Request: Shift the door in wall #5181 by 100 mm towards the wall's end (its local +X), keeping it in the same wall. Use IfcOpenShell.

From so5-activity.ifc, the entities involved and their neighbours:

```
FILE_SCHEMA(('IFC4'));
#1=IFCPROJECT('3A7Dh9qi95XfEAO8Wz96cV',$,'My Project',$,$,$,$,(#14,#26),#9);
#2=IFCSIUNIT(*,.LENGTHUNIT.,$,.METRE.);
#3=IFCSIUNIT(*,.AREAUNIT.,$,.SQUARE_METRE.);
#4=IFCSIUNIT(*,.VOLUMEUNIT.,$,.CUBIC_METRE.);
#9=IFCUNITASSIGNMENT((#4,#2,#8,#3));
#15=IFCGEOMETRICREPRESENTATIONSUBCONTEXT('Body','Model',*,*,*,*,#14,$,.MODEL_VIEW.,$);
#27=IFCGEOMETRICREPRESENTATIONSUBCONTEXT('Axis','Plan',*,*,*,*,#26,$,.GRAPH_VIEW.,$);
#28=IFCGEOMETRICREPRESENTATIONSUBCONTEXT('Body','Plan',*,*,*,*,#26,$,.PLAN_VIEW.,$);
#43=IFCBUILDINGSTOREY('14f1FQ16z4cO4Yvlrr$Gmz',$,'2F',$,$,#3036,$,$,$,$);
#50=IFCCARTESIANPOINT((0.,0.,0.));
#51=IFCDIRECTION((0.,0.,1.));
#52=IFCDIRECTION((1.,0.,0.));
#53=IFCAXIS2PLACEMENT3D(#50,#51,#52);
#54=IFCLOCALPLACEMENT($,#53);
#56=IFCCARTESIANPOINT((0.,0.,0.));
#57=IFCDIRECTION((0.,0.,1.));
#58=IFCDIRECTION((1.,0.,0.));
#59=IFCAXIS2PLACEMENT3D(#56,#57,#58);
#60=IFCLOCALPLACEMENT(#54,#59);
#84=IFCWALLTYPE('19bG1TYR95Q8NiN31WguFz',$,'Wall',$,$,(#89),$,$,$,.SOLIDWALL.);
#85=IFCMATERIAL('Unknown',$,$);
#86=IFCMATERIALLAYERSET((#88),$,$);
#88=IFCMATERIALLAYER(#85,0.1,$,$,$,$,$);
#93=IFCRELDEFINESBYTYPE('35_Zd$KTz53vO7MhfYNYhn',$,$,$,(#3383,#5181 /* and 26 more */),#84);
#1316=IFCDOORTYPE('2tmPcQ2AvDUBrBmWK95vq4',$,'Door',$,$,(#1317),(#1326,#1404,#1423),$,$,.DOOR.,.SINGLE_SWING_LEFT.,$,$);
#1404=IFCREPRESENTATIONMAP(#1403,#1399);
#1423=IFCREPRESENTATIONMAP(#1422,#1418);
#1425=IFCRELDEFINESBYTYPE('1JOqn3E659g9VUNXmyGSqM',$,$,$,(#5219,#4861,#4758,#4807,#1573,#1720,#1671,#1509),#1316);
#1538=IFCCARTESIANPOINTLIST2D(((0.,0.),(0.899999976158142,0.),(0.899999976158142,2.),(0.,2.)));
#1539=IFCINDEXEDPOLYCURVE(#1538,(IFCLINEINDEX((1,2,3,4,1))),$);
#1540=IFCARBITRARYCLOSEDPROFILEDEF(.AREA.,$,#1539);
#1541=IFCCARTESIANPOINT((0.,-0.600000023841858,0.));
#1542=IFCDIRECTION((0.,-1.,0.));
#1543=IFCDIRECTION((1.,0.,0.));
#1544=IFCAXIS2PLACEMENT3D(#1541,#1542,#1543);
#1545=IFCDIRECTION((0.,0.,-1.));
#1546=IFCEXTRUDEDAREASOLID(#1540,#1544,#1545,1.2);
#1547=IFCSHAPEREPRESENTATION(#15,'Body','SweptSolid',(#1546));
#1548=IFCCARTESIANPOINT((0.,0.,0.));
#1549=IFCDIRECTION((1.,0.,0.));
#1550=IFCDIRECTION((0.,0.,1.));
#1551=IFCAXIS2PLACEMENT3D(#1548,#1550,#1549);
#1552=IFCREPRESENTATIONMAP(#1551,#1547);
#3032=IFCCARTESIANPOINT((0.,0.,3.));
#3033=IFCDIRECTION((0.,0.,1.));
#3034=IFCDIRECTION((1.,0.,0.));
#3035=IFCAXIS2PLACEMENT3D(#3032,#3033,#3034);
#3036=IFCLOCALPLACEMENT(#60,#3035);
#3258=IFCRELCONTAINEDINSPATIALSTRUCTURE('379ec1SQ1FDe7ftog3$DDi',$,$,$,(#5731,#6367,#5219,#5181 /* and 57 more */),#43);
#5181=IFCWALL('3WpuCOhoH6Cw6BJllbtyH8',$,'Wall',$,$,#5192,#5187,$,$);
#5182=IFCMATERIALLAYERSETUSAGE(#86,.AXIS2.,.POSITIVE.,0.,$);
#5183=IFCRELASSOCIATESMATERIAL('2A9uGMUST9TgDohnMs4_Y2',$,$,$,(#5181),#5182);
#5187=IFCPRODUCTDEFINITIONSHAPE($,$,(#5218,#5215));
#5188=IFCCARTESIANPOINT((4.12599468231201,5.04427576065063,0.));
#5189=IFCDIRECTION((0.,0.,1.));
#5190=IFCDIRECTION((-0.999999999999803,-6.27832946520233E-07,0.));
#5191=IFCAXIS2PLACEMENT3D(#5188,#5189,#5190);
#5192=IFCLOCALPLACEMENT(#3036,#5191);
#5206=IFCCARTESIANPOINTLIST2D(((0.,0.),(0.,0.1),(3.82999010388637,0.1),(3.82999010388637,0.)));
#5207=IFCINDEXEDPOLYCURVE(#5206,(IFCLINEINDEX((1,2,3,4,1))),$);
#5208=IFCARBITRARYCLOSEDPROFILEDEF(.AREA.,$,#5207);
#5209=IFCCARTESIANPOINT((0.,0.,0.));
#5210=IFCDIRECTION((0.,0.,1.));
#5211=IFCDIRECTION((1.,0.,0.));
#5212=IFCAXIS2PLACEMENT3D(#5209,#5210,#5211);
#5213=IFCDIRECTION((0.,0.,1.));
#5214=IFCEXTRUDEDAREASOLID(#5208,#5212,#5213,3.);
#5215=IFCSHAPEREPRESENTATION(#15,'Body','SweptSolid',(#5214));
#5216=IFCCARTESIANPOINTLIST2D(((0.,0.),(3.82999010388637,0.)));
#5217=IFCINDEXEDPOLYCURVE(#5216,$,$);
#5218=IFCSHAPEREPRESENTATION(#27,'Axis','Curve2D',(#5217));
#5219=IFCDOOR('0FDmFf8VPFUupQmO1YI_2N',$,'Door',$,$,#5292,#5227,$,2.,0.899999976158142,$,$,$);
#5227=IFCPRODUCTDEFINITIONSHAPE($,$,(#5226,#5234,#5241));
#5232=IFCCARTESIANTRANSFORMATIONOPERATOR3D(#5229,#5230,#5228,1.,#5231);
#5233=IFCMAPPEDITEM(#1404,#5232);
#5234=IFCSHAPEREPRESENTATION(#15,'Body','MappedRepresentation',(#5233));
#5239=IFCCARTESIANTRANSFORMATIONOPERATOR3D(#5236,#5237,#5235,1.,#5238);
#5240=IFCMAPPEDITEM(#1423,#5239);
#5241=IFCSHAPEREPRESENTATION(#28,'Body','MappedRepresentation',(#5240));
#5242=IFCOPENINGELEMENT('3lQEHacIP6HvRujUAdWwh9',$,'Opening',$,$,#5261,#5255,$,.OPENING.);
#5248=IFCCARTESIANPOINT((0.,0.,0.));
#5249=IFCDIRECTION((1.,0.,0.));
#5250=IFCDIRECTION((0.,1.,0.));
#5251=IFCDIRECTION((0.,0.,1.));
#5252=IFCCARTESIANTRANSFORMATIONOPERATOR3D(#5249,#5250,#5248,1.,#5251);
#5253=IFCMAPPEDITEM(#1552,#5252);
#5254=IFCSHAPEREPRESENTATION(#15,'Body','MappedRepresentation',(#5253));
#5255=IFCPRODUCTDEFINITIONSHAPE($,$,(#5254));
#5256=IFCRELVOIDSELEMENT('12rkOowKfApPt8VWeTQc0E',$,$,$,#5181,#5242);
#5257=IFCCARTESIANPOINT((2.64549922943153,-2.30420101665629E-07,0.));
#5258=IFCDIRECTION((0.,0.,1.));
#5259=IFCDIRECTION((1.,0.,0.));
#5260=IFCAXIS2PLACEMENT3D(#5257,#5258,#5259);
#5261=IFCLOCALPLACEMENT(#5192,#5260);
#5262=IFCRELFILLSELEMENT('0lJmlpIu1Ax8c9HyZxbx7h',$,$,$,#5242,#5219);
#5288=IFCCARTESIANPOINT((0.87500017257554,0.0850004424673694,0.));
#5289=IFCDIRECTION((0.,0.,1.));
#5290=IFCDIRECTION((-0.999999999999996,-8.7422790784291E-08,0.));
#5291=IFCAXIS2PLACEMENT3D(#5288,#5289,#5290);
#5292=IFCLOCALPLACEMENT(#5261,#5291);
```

```python
import ifcopenshell
import ifcopenshell.api.geometry
import ifcopenshell.util.placement
import ifcopenshell.util.unit

model = ifcopenshell.open("so5-activity.ifc")
unit_scale = ifcopenshell.util.unit.calculate_unit_scale(model)

door = model.by_guid("0FDmFf8VPFUupQmO1YI_2N")
opening = door.FillsVoids[0].RelatingOpeningElement
wall = opening.VoidsElements[0].RelatingBuildingElement

wall_matrix = ifcopenshell.util.placement.get_local_placement(wall.ObjectPlacement)
shift = wall_matrix[:3, 0] * 0.1 / unit_scale
before = ifcopenshell.util.placement.get_local_placement(door.ObjectPlacement)[:3, 3].copy()

# The door is placed relative to its opening, so it follows when the opening moves.
matrix = ifcopenshell.util.placement.get_local_placement(opening.ObjectPlacement)
matrix[:3, 3] += shift
ifcopenshell.api.geometry.edit_object_placement(
    model, product=opening, matrix=matrix, is_si=False, should_transform_children=True
)

after = ifcopenshell.util.placement.get_local_placement(door.ObjectPlacement)[:3, 3]
print("door moved by", (after - before).round(3) + 0.0)

model.write("so5-activity_v2.ifc")
```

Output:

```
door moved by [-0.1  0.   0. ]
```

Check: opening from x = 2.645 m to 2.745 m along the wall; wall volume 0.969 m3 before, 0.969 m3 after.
